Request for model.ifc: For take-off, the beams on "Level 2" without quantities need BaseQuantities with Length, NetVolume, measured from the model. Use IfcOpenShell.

First a look at what the model holds.

```python
import ifcopenshell
import ifcopenshell.util.element
import ifcopenshell.util.unit

model = ifcopenshell.open("model.ifc")
print(model.schema)
for unit_type in ("LENGTHUNIT", "AREAUNIT", "VOLUMEUNIT"):
    print(unit_type, ifcopenshell.util.unit.calculate_unit_scale(model, unit_type))
storey = next(s for s in model.by_type("IfcBuildingStorey") if s.Name == "Level 2")
beams = [e for e in ifcopenshell.util.element.get_decomposition(storey) if e.is_a("IfcBeam")]
for e in sorted(beams, key=lambda e: e.id()):
    print(e.id(), e.is_a(), e.Name, list(ifcopenshell.util.element.get_psets(e, qtos_only=True)), sep=" | ")
```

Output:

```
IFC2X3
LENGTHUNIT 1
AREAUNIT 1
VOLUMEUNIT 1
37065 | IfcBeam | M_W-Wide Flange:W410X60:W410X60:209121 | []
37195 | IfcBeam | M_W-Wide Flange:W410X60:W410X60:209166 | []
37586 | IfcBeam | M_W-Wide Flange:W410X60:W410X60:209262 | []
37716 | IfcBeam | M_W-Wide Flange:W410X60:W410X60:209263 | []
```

```python
import ifcopenshell
import ifcopenshell.api.pset
import ifcopenshell.geom
import ifcopenshell.util.element
import ifcopenshell.util.shape
import ifcopenshell.util.unit

model = ifcopenshell.open("model.ifc")
unit_scale = ifcopenshell.util.unit.calculate_unit_scale(model)
volume_scale = ifcopenshell.util.unit.calculate_unit_scale(model, "VOLUMEUNIT")
settings = ifcopenshell.geom.settings()

storey = next(s for s in model.by_type("IfcBuildingStorey") if s.Name == "Level 2")
beams = [e for e in ifcopenshell.util.element.get_decomposition(storey) if e.is_a("IfcBeam")]

for e in sorted(beams, key=lambda e: e.id()):
    if ifcopenshell.util.element.get_psets(e, qtos_only=True, should_inherit=False):
        continue
    # Geometry comes back in metres, in the element's own axes.
    shape = ifcopenshell.geom.create_shape(settings, e)
    values = {
        "Length": ifcopenshell.util.shape.get_max_xyz(shape.geometry) / unit_scale,
        "NetVolume": ifcopenshell.util.shape.get_volume(shape.geometry) / volume_scale,
    }
    qto = ifcopenshell.api.pset.add_qto(model, product=e, name="BaseQuantities")
    ifcopenshell.api.pset.edit_qto(model, qto=qto, properties=values)
    print(e.id(), {k: round(v, 3) for k, v in values.items()})

model.write("model_updated.ifc")
```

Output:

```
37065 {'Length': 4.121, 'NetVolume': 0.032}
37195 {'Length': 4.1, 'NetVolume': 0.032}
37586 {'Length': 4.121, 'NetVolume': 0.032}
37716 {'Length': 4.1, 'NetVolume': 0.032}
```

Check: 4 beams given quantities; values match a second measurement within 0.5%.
